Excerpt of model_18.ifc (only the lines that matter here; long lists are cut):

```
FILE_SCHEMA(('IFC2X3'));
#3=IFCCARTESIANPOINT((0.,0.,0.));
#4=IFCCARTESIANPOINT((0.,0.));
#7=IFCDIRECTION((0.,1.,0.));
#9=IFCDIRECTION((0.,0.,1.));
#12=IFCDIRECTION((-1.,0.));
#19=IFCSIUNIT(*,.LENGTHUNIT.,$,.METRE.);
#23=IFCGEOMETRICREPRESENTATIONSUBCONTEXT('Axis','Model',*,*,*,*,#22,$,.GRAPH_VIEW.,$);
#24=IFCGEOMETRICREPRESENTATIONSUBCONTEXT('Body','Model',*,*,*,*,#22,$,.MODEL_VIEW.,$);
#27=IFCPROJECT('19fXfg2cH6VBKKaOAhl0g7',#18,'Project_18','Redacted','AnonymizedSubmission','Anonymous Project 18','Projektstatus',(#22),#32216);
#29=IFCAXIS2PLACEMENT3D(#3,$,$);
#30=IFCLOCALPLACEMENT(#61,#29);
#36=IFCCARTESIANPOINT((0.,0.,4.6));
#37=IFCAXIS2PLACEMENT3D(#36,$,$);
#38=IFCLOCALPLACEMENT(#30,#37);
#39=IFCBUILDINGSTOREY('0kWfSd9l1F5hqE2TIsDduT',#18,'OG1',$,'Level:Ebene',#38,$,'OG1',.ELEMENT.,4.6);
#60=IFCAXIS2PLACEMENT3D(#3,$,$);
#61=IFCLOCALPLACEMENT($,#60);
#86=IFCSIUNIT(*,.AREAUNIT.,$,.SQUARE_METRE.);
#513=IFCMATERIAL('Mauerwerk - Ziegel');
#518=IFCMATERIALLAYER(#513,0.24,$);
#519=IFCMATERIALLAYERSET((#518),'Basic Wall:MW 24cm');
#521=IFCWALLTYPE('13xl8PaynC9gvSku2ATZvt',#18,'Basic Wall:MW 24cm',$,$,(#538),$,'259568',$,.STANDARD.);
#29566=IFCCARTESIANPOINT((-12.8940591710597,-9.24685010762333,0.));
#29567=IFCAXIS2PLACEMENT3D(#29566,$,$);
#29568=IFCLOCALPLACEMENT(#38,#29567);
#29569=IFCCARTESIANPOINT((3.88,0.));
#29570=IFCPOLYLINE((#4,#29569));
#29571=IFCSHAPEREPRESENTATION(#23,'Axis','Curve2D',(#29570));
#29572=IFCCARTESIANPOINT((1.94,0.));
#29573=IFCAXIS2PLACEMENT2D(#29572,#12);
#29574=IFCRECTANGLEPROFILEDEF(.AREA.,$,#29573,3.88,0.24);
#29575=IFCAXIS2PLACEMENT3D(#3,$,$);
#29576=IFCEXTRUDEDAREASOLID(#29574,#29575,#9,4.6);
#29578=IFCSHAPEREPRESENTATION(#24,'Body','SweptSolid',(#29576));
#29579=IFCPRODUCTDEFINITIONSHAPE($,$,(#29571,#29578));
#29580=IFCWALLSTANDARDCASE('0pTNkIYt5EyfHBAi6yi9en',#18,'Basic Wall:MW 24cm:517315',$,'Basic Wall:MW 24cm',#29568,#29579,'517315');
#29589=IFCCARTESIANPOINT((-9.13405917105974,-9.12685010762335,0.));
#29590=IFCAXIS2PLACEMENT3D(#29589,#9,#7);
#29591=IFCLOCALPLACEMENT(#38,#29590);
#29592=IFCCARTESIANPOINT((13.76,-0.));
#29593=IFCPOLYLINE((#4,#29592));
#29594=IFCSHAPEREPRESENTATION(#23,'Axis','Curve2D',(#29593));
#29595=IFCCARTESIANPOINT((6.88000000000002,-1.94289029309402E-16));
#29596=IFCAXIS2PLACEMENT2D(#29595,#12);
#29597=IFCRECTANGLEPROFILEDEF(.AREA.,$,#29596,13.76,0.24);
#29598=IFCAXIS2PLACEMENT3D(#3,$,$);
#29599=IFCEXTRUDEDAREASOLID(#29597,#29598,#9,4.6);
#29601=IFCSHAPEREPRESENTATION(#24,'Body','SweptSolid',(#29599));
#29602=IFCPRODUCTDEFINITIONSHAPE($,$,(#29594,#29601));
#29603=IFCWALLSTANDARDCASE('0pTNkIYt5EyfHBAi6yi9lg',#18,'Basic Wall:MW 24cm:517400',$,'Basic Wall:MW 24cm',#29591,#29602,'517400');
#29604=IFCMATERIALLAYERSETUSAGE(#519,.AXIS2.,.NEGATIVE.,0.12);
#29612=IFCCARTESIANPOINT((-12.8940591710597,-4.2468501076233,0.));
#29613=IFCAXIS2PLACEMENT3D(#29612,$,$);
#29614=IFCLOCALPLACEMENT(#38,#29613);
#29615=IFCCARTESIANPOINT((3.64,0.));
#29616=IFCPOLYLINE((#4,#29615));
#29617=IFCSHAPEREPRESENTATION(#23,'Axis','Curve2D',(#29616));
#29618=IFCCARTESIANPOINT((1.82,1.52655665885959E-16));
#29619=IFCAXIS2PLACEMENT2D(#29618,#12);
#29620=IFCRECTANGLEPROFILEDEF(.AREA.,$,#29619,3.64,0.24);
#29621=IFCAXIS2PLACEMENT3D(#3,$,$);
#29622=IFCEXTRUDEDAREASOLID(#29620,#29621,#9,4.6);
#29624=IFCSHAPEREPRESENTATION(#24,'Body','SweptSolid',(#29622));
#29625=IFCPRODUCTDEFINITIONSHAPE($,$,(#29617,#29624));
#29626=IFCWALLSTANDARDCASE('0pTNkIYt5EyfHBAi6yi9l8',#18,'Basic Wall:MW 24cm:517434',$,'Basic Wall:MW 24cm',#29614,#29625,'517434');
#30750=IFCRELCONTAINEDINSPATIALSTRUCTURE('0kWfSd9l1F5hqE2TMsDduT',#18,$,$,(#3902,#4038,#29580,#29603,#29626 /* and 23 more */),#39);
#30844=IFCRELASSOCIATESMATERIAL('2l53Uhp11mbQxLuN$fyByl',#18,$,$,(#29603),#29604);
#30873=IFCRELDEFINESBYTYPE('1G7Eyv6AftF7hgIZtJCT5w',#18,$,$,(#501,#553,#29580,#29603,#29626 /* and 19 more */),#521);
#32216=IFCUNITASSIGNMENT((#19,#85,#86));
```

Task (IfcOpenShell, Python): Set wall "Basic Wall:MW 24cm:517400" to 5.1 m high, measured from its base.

```python
import ifcopenshell
import ifcopenshell.geom
import ifcopenshell.util.representation
import ifcopenshell.util.shape

model = ifcopenshell.open("model_18.ifc")
settings = ifcopenshell.geom.settings()


def volume(element):
    """Net volume in cubic metres, openings subtracted."""
    shape = ifcopenshell.geom.create_shape(settings, element)
    return ifcopenshell.util.shape.get_volume(shape.geometry)


wall = model.by_guid("0pTNkIYt5EyfHBAi6yi9lg")
before = volume(wall)

body = ifcopenshell.util.representation.get_representation(wall, "Model", "Body")
solid = body.Items[0]
old_height = solid.Depth
solid.Depth = 5.1
after = volume(wall)

print(f"height {old_height:g} -> {solid.Depth:g}, volume {before:.3f} -> {after:.3f} m3")

model.write("model_18-out.ifc")
```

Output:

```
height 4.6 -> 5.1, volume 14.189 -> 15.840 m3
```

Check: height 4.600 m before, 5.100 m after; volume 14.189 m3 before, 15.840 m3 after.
